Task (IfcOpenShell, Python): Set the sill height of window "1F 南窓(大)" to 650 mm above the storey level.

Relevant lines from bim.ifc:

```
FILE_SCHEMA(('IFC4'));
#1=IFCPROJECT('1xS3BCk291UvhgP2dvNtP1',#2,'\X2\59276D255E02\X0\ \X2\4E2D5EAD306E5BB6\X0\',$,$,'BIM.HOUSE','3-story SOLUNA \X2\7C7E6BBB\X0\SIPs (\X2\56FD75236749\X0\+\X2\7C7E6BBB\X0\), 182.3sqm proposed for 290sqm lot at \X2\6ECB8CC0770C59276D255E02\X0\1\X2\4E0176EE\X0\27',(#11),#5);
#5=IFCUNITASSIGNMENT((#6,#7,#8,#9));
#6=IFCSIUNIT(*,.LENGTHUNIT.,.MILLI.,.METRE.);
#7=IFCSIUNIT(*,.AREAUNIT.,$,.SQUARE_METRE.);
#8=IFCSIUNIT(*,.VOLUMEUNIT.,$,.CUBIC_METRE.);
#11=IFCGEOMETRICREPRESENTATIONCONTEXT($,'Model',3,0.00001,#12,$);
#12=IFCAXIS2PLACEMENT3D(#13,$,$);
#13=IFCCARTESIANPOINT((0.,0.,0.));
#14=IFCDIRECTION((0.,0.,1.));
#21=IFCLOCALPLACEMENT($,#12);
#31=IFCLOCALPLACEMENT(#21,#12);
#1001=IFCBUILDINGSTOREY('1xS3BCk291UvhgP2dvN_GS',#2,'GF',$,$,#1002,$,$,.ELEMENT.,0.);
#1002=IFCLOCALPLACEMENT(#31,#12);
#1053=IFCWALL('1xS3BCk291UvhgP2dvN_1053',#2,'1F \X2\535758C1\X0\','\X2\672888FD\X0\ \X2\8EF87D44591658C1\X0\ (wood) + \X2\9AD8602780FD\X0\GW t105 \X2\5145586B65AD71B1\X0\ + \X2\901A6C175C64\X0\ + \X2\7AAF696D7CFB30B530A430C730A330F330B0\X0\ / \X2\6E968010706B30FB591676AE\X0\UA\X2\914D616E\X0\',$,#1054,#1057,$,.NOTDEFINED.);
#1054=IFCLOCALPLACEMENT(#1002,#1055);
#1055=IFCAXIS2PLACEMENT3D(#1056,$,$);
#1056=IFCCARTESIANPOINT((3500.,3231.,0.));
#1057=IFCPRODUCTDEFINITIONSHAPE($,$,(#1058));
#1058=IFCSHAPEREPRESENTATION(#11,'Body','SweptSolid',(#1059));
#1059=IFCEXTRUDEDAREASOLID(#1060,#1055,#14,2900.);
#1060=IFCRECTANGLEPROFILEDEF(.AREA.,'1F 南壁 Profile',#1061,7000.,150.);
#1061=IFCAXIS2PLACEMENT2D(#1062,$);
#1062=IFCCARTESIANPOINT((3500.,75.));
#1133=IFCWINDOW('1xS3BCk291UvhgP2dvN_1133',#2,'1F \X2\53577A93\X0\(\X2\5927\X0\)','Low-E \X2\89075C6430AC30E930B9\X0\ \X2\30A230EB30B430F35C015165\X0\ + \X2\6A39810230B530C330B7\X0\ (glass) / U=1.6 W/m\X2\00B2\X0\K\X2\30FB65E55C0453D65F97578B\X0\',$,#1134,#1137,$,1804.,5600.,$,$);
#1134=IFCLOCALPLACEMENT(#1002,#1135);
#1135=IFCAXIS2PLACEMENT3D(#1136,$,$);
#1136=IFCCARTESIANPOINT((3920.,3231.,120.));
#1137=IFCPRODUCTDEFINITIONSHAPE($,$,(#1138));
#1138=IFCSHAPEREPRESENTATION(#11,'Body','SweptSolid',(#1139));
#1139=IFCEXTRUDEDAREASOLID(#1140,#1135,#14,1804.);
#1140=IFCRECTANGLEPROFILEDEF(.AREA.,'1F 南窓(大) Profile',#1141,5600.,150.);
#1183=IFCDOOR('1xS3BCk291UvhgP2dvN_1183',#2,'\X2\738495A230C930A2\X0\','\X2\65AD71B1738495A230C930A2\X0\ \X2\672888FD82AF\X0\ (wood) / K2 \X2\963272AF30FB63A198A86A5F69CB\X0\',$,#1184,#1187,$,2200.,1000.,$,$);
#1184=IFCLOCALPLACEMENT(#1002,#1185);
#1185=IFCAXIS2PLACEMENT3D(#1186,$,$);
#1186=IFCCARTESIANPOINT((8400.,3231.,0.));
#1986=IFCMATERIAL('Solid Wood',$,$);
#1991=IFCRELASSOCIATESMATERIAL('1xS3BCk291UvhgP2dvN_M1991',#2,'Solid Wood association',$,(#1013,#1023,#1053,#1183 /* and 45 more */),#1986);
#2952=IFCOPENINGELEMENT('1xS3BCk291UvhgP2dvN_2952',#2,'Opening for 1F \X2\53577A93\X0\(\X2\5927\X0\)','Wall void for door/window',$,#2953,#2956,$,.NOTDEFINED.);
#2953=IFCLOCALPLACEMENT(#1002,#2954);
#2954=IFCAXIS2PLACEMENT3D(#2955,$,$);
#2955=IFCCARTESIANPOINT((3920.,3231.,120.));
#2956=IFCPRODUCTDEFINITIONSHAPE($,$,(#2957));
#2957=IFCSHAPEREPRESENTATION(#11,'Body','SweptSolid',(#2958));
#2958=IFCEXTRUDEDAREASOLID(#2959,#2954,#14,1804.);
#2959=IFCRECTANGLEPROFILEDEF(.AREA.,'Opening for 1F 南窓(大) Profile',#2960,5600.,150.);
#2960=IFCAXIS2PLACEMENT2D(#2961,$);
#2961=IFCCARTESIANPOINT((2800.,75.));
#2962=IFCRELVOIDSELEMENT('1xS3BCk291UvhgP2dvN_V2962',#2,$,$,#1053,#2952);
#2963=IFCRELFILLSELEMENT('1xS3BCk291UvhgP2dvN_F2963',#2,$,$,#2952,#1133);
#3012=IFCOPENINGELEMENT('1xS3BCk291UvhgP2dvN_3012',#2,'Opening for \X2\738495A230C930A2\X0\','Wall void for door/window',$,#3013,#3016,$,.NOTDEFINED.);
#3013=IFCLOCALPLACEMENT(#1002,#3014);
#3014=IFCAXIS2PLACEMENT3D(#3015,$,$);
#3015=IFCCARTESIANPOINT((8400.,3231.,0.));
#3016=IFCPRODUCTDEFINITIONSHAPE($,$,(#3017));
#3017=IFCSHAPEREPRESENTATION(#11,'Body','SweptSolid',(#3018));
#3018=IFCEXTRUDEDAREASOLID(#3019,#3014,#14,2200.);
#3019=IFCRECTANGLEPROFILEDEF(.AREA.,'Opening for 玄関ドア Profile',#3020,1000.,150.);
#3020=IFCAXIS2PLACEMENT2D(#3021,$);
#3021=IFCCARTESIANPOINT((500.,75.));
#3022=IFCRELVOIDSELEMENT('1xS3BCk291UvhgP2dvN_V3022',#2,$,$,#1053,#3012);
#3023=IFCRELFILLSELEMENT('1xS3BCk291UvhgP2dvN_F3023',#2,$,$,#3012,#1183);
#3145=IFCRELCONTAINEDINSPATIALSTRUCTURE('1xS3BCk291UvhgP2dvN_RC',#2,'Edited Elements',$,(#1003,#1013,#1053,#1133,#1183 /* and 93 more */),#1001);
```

```python
import numpy as np
import ifcopenshell
import ifcopenshell.api.geometry
import ifcopenshell.geom
import ifcopenshell.util.element
import ifcopenshell.util.placement
import ifcopenshell.util.shape
import ifcopenshell.util.unit

model = ifcopenshell.open("bim.ifc")
unit_scale = ifcopenshell.util.unit.calculate_unit_scale(model)

window = model.by_id(1133)
opening = window.FillsVoids[0].RelatingOpeningElement
storey = ifcopenshell.util.element.get_container(window, ifc_class="IfcBuildingStorey")
level = ifcopenshell.util.placement.get_local_placement(storey.ObjectPlacement)[2, 3]

# The opening's origin need not be at the sill, so measure its lowest point.
shape = ifcopenshell.geom.create_shape(ifcopenshell.geom.settings(), opening)
bottom = ifcopenshell.util.shape.get_shape_bottom_elevation(shape, shape.geometry) / unit_scale
dz = level + 0.65 / unit_scale - bottom

shift = np.array([0.0, 0.0, dz])
# The window is not placed relative to its opening, so move both.
for product in (opening, window):
    matrix = ifcopenshell.util.placement.get_local_placement(product.ObjectPlacement)
    matrix[:3, 3] += shift
    ifcopenshell.api.geometry.edit_object_placement(model, product=product, matrix=matrix, is_si=False)

print(f"moved by {dz * unit_scale:+.3f} m")

model.write("bim-out.ifc")
```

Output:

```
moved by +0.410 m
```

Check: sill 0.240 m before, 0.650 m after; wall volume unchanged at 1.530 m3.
